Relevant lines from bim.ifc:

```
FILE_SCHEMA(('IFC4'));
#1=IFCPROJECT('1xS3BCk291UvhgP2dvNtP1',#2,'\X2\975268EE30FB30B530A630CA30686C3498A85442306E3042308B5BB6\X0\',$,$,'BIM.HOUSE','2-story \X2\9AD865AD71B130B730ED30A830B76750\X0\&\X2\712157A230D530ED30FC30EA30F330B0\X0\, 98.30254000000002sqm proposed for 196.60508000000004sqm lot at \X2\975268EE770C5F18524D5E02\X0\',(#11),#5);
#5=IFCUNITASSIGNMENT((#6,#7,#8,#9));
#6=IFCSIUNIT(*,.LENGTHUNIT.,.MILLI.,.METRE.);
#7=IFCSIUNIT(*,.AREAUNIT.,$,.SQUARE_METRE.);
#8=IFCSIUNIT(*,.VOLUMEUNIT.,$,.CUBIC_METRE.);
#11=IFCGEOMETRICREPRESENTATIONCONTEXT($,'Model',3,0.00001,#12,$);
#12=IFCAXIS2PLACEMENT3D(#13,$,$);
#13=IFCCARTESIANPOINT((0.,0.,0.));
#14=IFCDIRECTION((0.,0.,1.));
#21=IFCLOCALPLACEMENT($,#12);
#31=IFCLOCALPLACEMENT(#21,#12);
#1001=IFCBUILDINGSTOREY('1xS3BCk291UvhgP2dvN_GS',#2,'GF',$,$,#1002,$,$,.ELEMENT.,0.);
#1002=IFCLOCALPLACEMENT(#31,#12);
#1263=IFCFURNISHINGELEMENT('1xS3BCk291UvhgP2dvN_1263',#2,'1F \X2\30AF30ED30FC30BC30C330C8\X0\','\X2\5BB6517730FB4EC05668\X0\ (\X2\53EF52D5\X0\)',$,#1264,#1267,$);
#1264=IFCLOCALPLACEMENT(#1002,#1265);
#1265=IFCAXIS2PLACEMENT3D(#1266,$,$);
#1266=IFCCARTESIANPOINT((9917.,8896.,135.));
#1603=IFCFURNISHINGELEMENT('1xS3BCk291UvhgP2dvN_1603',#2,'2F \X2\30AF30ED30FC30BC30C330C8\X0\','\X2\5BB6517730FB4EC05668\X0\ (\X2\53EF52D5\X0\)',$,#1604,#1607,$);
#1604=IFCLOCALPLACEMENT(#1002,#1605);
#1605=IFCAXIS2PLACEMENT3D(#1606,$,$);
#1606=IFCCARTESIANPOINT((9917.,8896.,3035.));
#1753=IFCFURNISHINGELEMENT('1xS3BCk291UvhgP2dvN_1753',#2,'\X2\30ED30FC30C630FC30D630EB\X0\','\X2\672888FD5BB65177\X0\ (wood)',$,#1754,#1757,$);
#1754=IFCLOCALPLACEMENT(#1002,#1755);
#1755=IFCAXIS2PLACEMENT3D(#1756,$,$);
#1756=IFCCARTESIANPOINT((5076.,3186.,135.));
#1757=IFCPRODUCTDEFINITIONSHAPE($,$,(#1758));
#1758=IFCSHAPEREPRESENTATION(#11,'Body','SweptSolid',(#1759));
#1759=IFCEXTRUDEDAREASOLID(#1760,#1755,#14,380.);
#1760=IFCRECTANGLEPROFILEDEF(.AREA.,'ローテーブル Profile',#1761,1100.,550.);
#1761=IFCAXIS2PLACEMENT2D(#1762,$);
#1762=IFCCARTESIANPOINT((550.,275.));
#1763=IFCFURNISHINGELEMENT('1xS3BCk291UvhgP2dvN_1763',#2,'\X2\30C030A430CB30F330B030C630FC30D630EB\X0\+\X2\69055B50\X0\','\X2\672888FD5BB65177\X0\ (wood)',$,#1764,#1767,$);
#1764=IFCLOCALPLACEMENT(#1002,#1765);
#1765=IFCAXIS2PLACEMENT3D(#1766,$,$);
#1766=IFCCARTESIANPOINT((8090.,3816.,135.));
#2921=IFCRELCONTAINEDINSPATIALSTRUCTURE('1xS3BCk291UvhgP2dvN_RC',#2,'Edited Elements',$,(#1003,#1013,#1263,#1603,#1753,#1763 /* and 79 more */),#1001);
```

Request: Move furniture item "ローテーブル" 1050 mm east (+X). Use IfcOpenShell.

```python
import ifcopenshell
import ifcopenshell.api.geometry
import ifcopenshell.util.placement

model = ifcopenshell.open("bim.ifc")

item = model.by_id(1753)
matrix = ifcopenshell.util.placement.get_local_placement(item.ObjectPlacement)
matrix[0, 3] += 1050.0
ifcopenshell.api.geometry.edit_object_placement(model, product=item, matrix=matrix, is_si=False)

print(ifcopenshell.util.placement.get_local_placement(item.ObjectPlacement).round(3) + 0.0)

model.write("bim-out.ifc")
```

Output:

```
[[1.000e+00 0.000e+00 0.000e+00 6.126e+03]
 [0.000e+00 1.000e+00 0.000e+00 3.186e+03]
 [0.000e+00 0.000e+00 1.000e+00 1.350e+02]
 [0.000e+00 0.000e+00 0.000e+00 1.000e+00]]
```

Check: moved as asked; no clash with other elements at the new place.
